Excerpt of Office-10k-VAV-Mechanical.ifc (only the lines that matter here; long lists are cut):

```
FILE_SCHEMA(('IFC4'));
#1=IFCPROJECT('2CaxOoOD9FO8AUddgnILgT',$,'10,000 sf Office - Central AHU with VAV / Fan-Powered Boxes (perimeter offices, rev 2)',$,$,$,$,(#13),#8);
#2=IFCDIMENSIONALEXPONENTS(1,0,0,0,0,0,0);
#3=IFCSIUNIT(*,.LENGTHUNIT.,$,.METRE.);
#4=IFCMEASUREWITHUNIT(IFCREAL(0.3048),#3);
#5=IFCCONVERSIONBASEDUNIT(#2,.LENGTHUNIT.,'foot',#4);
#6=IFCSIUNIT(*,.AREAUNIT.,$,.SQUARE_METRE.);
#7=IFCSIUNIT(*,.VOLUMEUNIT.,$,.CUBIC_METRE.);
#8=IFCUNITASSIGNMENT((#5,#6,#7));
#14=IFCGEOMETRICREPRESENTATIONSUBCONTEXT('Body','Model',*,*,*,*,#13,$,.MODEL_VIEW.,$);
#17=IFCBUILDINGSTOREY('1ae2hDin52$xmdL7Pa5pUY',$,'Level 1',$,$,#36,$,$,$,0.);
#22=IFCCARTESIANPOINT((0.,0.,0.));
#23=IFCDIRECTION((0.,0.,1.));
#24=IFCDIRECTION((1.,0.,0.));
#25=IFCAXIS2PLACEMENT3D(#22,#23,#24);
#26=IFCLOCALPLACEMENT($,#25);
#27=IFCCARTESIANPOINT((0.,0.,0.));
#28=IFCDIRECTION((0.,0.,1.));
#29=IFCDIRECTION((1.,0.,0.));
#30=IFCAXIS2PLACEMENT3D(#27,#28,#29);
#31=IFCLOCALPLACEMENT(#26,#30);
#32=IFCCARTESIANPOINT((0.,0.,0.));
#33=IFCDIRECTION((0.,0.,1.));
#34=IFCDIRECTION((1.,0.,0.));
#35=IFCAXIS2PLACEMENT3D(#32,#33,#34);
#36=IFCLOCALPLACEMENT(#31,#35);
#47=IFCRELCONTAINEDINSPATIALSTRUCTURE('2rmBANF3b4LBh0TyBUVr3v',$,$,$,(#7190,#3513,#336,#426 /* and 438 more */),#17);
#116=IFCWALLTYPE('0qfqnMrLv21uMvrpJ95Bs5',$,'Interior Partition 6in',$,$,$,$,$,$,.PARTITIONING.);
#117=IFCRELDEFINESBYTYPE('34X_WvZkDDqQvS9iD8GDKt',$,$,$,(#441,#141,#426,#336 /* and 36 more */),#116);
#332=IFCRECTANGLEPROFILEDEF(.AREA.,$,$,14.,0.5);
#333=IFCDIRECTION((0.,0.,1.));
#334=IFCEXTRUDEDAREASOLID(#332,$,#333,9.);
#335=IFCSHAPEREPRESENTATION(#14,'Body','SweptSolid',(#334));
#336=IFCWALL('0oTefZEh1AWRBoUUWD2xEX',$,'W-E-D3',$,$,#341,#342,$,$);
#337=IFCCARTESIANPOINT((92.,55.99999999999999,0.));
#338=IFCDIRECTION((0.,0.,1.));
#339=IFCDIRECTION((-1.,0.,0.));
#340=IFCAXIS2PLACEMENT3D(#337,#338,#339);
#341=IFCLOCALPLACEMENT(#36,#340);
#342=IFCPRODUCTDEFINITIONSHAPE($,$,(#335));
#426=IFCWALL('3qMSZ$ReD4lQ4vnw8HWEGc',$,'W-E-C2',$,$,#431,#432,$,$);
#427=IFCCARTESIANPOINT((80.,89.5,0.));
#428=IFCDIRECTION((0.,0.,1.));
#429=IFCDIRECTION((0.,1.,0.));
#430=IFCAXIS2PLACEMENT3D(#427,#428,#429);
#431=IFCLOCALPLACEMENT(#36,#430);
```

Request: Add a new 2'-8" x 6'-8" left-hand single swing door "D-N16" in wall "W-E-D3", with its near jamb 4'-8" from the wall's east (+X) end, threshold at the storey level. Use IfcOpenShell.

```python
import numpy as np
import ifcopenshell
import ifcopenshell.api.feature
import ifcopenshell.api.geometry
import ifcopenshell.api.root
import ifcopenshell.api.spatial
import ifcopenshell.geom
import ifcopenshell.util.element
import ifcopenshell.util.placement
import ifcopenshell.util.representation
import ifcopenshell.util.shape
import ifcopenshell.util.unit

model = ifcopenshell.open("Office-10k-VAV-Mechanical.ifc")
unit_scale = ifcopenshell.util.unit.calculate_unit_scale(model)
settings = ifcopenshell.geom.settings()


def volume(element):
    """Net volume in cubic metres, openings subtracted."""
    shape = ifcopenshell.geom.create_shape(settings, element)
    return ifcopenshell.util.shape.get_volume(shape.geometry)


wall = model.by_guid("0oTefZEh1AWRBoUUWD2xEX")
storey = ifcopenshell.util.element.get_container(wall, ifc_class="IfcBuildingStorey")
context = ifcopenshell.util.representation.get_context(model, "Model", "Body", "MODEL_VIEW")
before = volume(wall)

width, height, from_end, sill = 0.8128, 2.032, 1.4224, 0.0  # metres

# The wall runs along its own X axis, and the end named is its -X end.
wall_shape = ifcopenshell.geom.create_shape(settings, wall)
x, y, z = ifcopenshell.util.shape.get_vertices(wall_shape.geometry).T
start = x.min() + from_end
face, thickness = float(y.min()), float(y.max() - y.min())
wall_matrix = ifcopenshell.util.placement.get_local_placement(wall.ObjectPlacement)
level = ifcopenshell.util.placement.get_local_placement(storey.ObjectPlacement)[2, 3]


def in_wall(x, y):
    """Placement at x, y metres in the wall's axes, at sill height."""
    matrix = wall_matrix.copy()
    matrix[:, 3] = wall_matrix @ np.array([x / unit_scale, y / unit_scale, 0.0, 1.0])
    matrix[2, 3] = level + sill / unit_scale
    return matrix


# Opening: a box that overshoots both wall faces by 50 mm.
opening = ifcopenshell.api.root.create_entity(model, ifc_class="IfcOpeningElement", predefined_type="OPENING")
box = ifcopenshell.api.geometry.add_wall_representation(
    model, context=context, length=width, height=height, thickness=thickness + 0.1
)
ifcopenshell.api.geometry.assign_representation(model, product=opening, representation=box)
ifcopenshell.api.geometry.edit_object_placement(model, product=opening, matrix=in_wall(start, face - 0.05), is_si=False)
ifcopenshell.api.feature.add_feature(model, feature=opening, element=wall)

door = ifcopenshell.api.root.create_entity(model, ifc_class="IfcDoor", name="D-N16", predefined_type="DOOR")
door.OverallWidth, door.OverallHeight = width / unit_scale, height / unit_scale
door.OperationType = "SINGLE_SWING_LEFT"
body = ifcopenshell.api.geometry.add_door_representation(
    model,
    context=context,
    overall_width=door.OverallWidth,
    overall_height=door.OverallHeight,
    operation_type="SINGLE_SWING_LEFT",
    lining_properties={"LiningDepth": thickness / unit_scale, "ThresholdDepth": thickness / unit_scale},
)
ifcopenshell.api.geometry.assign_representation(model, product=door, representation=body)
ifcopenshell.api.spatial.assign_container(model, products=[door], relating_structure=storey)
ifcopenshell.api.feature.add_filling(model, opening=opening, element=door)

# The lining spans the wall, so the door starts at the wall face.
ifcopenshell.api.geometry.edit_object_placement(model, product=door, matrix=in_wall(start, face), is_si=False)

after = volume(wall)

print(f"wall volume {before:.3f} -> {after:.3f} m3")

model.write("Office-10k-VAV-Mechanical_v2.ifc")
```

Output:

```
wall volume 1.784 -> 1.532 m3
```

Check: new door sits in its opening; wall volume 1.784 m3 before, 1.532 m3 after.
